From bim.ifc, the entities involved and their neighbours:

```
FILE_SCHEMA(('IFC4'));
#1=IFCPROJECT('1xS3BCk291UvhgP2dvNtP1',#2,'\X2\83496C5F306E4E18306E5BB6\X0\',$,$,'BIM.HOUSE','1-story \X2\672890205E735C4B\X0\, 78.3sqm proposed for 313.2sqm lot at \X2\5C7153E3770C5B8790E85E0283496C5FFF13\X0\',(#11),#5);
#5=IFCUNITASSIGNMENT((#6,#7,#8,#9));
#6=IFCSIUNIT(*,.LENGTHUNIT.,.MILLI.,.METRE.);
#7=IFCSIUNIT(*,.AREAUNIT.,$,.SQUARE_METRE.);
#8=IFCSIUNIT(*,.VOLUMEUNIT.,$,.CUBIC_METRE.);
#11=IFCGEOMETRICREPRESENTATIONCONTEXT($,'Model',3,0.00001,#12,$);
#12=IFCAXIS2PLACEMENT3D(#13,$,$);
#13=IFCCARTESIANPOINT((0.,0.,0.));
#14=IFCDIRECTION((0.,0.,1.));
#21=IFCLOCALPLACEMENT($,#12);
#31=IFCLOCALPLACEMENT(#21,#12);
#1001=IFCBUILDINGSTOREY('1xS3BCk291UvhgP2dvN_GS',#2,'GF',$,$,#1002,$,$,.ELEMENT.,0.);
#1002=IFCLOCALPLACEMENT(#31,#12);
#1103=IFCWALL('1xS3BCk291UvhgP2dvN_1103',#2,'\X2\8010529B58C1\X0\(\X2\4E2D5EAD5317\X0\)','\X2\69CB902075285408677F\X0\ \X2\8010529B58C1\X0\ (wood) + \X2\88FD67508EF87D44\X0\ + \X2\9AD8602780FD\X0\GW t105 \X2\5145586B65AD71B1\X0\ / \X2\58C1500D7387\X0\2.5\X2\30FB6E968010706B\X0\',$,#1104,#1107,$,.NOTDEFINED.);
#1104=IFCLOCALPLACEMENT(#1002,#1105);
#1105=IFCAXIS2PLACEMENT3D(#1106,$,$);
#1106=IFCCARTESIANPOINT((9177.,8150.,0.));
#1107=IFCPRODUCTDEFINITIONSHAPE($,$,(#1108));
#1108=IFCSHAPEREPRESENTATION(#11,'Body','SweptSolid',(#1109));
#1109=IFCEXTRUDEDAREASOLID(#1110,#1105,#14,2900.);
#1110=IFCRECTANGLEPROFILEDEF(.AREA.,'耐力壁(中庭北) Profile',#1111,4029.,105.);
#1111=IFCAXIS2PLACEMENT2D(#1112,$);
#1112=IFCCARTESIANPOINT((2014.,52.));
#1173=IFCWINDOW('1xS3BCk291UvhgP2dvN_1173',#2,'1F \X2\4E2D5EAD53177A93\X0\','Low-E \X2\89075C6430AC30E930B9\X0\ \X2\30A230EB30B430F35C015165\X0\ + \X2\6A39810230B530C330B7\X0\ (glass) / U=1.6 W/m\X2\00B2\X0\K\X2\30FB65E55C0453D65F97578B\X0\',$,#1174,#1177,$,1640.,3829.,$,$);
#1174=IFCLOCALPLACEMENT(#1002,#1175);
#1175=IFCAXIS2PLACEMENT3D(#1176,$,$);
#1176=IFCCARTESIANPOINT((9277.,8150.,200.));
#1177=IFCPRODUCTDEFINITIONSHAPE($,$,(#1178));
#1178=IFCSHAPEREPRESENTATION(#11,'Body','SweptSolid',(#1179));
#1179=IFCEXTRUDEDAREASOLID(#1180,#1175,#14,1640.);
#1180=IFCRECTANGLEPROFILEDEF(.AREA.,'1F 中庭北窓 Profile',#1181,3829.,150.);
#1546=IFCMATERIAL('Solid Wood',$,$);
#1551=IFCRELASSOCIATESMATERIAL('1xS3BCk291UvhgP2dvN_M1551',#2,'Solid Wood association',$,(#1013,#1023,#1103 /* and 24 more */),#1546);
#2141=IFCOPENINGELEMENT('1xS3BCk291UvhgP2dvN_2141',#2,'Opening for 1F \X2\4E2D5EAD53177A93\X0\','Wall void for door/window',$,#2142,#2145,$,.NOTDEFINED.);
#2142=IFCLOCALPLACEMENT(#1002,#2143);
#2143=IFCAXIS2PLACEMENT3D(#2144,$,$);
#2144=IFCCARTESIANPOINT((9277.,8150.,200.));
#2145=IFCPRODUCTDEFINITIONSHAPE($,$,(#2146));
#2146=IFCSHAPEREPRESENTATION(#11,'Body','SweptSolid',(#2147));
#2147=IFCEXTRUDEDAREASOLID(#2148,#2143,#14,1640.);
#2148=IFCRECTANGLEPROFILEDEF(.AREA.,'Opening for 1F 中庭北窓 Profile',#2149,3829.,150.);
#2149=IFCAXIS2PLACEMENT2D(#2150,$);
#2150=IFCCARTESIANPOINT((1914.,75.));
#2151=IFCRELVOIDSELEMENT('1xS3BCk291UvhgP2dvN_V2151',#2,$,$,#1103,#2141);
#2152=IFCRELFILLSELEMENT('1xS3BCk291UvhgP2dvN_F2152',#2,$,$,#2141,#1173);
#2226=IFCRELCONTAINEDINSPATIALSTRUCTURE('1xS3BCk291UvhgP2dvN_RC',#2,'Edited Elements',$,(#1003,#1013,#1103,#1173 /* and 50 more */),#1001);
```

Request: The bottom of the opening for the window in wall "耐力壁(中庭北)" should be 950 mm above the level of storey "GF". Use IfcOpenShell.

```python
import numpy as np
import ifcopenshell
import ifcopenshell.api.geometry
import ifcopenshell.geom
import ifcopenshell.util.element
import ifcopenshell.util.placement
import ifcopenshell.util.shape
import ifcopenshell.util.unit

model = ifcopenshell.open("bim.ifc")
unit_scale = ifcopenshell.util.unit.calculate_unit_scale(model)

window = model.by_id(1173)
opening = window.FillsVoids[0].RelatingOpeningElement
storey = ifcopenshell.util.element.get_container(window, ifc_class="IfcBuildingStorey")
level = ifcopenshell.util.placement.get_local_placement(storey.ObjectPlacement)[2, 3]

# The opening's origin need not be at the sill, so measure its lowest point.
shape = ifcopenshell.geom.create_shape(ifcopenshell.geom.settings(), opening)
bottom = ifcopenshell.util.shape.get_shape_bottom_elevation(shape, shape.geometry) / unit_scale
dz = level + 0.95 / unit_scale - bottom

shift = np.array([0.0, 0.0, dz])
# The window is not placed relative to its opening, so move both.
for product in (opening, window):
    matrix = ifcopenshell.util.placement.get_local_placement(product.ObjectPlacement)
    matrix[:3, 3] += shift
    ifcopenshell.api.geometry.edit_object_placement(model, product=product, matrix=matrix, is_si=False)

print(f"moved by {dz * unit_scale:+.3f} m")

model.write("bim_rev.ifc")
```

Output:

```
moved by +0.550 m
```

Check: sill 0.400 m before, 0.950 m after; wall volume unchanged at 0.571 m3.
